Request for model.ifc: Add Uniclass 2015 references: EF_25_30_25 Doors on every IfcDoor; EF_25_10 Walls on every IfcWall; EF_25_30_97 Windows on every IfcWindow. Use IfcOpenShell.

First a look at what the model holds.

```python
import ifcopenshell

model = ifcopenshell.open("model.ifc")
print(model.schema)
print("classifications:", [c.Name for c in model.by_type("IfcClassification")])
for ifc_class in ("IfcDoor", "IfcRoof", "IfcStair", "IfcWall", "IfcWindow"):
    print(ifc_class, len(model.by_type(ifc_class)))
```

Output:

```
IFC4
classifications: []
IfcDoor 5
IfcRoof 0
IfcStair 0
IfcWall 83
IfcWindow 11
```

```python
import ifcopenshell
import ifcopenshell.api.classification

model = ifcopenshell.open("model.ifc")

system = ifcopenshell.api.classification.add_classification(model, classification="Uniclass 2015")

codes = {
    "IfcDoor": ("EF_25_30_25", "Doors"),
    "IfcWall": ("EF_25_10", "Walls"),
    "IfcWindow": ("EF_25_30_97", "Windows"),
}
for ifc_class, (code, name) in codes.items():
    products = model.by_type(ifc_class)
    ifcopenshell.api.classification.add_reference(
        model, products=products, classification=system, identification=code, name=name
    )
    print(code, len(products))

model.write("model_updated.ifc")
```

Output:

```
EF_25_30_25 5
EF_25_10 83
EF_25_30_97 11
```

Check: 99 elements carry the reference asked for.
